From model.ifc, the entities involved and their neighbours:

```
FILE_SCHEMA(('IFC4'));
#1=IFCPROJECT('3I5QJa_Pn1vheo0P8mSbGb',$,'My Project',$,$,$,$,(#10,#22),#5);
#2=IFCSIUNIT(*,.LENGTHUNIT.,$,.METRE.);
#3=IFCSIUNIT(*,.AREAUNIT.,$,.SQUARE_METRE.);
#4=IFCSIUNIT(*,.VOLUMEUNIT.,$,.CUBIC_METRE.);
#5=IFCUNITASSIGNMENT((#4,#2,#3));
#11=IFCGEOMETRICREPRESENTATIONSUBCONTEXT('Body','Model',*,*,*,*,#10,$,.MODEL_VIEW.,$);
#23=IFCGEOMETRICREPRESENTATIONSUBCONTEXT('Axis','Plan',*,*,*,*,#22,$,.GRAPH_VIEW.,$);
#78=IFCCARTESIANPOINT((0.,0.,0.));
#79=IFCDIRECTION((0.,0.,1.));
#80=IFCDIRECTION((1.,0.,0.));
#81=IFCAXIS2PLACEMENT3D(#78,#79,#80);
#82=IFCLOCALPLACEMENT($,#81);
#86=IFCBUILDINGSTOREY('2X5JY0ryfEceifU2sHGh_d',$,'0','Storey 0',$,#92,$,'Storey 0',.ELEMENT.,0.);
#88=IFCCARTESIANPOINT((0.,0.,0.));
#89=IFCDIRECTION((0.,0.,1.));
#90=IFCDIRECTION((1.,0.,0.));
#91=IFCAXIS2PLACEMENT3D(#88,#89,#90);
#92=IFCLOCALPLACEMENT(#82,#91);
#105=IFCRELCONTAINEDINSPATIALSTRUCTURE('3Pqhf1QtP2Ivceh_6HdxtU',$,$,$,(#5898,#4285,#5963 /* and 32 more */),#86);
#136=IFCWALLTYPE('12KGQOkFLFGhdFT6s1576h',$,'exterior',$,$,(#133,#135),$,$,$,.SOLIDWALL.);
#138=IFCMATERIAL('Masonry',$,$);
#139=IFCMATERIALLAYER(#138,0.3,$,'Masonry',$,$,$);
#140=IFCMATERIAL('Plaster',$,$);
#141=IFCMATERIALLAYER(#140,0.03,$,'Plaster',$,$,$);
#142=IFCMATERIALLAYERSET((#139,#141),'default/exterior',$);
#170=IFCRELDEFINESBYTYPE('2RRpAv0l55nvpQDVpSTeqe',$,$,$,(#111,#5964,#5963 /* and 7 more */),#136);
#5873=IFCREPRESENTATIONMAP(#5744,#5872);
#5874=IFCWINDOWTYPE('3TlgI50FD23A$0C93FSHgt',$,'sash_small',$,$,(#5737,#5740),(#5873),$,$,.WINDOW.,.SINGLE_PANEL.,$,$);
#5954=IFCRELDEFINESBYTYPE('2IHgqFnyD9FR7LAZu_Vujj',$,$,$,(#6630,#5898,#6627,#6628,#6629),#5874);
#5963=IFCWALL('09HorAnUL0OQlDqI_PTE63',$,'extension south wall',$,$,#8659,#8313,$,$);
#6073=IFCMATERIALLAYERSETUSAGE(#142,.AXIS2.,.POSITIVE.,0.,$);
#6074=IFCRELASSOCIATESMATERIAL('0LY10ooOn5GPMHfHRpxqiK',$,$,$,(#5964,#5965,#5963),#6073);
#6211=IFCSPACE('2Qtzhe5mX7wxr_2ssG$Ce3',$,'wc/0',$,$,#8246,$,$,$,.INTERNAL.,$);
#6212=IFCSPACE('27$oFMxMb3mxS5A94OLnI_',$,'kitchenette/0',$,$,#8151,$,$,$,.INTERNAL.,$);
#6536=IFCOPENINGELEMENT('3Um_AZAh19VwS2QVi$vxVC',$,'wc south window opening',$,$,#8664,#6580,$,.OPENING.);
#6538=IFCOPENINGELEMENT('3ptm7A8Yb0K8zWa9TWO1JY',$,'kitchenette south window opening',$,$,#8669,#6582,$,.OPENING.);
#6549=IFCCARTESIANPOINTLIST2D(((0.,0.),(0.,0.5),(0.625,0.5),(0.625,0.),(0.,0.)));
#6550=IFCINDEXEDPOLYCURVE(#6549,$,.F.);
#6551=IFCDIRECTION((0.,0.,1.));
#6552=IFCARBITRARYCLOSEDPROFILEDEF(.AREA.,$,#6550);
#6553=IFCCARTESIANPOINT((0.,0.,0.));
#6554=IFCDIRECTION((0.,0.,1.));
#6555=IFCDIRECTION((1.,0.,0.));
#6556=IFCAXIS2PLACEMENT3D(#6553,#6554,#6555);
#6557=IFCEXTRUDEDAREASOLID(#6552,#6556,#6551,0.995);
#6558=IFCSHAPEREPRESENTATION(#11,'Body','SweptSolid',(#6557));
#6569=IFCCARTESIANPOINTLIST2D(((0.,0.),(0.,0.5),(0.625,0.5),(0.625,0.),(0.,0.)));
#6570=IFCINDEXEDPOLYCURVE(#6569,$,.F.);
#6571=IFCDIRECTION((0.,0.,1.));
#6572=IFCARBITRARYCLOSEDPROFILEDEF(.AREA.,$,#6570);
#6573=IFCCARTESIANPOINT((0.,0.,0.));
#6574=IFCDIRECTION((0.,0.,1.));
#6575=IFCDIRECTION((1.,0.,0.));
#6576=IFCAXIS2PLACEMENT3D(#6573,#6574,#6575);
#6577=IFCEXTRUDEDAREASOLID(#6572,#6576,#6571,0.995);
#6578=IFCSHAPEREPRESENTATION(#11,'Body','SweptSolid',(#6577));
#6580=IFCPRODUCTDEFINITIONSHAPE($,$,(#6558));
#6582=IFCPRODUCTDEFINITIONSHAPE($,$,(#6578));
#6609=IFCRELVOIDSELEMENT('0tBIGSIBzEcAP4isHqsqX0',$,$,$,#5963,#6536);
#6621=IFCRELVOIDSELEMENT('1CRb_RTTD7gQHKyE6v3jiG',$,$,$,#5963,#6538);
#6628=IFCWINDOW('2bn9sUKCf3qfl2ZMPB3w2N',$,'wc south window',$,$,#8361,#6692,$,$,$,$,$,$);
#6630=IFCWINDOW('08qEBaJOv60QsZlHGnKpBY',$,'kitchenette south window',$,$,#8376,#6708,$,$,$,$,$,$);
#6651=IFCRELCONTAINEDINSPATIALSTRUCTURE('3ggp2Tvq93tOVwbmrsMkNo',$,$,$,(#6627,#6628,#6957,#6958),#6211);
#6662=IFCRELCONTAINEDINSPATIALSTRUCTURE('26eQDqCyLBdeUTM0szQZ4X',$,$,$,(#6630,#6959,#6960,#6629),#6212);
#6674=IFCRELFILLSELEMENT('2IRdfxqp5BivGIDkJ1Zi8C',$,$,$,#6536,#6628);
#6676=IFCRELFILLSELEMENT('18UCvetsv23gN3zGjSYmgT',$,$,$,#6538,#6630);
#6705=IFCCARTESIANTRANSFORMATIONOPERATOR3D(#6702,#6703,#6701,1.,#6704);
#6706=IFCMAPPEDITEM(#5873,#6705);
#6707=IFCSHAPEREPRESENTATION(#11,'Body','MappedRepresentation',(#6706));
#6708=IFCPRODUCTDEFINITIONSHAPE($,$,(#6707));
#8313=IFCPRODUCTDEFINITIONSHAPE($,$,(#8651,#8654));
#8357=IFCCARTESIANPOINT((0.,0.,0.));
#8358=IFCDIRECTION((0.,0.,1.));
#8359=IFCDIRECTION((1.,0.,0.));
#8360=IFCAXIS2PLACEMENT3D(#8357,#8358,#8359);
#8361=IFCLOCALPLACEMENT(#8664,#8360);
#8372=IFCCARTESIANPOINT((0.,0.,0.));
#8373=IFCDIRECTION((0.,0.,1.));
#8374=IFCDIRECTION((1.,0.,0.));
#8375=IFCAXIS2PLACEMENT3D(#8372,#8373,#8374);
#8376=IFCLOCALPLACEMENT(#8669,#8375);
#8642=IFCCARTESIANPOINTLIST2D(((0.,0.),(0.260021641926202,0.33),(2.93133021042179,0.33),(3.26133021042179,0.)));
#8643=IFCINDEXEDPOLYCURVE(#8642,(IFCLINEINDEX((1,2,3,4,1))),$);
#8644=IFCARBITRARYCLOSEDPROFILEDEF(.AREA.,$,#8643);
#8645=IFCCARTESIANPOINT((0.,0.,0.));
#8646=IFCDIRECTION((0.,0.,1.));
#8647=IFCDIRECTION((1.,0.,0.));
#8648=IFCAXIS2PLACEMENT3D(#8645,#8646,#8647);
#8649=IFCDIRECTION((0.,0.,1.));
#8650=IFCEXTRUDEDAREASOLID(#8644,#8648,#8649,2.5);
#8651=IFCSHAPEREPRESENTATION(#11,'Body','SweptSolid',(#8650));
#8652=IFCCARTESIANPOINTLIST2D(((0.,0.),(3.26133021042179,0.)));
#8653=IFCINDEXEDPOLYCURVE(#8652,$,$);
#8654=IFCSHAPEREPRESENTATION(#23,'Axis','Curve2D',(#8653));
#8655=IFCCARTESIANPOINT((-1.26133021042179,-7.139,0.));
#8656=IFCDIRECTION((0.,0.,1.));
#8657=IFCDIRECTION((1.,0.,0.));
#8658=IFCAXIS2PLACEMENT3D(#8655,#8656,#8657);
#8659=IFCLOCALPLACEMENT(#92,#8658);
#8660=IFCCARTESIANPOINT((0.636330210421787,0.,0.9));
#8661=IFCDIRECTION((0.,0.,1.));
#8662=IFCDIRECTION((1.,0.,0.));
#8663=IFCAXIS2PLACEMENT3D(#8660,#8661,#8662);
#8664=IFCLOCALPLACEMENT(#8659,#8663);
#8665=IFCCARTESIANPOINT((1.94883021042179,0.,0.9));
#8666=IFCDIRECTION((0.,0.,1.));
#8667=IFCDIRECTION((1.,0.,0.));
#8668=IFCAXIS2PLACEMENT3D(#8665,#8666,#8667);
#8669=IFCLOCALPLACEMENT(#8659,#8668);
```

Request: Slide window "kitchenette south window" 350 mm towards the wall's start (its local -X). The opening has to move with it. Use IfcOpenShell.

```python
import ifcopenshell
import ifcopenshell.api.geometry
import ifcopenshell.util.placement
import ifcopenshell.util.unit

model = ifcopenshell.open("model.ifc")
unit_scale = ifcopenshell.util.unit.calculate_unit_scale(model)

window = model.by_guid("08qEBaJOv60QsZlHGnKpBY")
opening = window.FillsVoids[0].RelatingOpeningElement
wall = opening.VoidsElements[0].RelatingBuildingElement

wall_matrix = ifcopenshell.util.placement.get_local_placement(wall.ObjectPlacement)
shift = wall_matrix[:3, 0] * -0.35 / unit_scale
before = ifcopenshell.util.placement.get_local_placement(window.ObjectPlacement)[:3, 3].copy()

# The window is placed relative to its opening, so it follows when the opening moves.
matrix = ifcopenshell.util.placement.get_local_placement(opening.ObjectPlacement)
matrix[:3, 3] += shift
ifcopenshell.api.geometry.edit_object_placement(
    model, product=opening, matrix=matrix, is_si=False, should_transform_children=True
)

after = ifcopenshell.util.placement.get_local_placement(window.ObjectPlacement)[:3, 3]
print("window moved by", (after - before).round(3) + 0.0)

model.write("model_updated.ifc")
```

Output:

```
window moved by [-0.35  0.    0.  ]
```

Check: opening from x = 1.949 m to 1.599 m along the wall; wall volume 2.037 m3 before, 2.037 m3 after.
